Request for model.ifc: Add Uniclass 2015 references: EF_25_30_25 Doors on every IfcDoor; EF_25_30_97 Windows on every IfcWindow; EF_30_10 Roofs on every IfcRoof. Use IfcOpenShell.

First a look at what the model holds.

```python
import ifcopenshell

model = ifcopenshell.open("model.ifc")
print(model.schema)
print("classifications:", [c.Name for c in model.by_type("IfcClassification")])
for ifc_class in ("IfcDoor", "IfcRoof", "IfcStair", "IfcWall", "IfcWindow"):
    print(ifc_class, len(model.by_type(ifc_class)))
```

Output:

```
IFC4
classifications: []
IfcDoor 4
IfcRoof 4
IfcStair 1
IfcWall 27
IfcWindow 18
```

```python
import ifcopenshell
import ifcopenshell.api.classification

model = ifcopenshell.open("model.ifc")

system = ifcopenshell.api.classification.add_classification(model, classification="Uniclass 2015")

codes = {
    "IfcDoor": ("EF_25_30_25", "Doors"),
    "IfcWindow": ("EF_25_30_97", "Windows"),
    "IfcRoof": ("EF_30_10", "Roofs"),
}
for ifc_class, (code, name) in codes.items():
    products = model.by_type(ifc_class)
    ifcopenshell.api.classification.add_reference(
        model, products=products, classification=system, identification=code, name=name
    )
    print(code, len(products))

model.write("model-out.ifc")
```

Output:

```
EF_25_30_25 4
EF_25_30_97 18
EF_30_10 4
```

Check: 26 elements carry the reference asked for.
